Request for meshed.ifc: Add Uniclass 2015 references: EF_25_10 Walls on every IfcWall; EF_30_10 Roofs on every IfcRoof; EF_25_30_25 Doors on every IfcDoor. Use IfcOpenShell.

First a look at what the model holds.

```python
import ifcopenshell

model = ifcopenshell.open("meshed.ifc")
print(model.schema)
print("classifications:", [c.Name for c in model.by_type("IfcClassification")])
for ifc_class in ("IfcDoor", "IfcRoof", "IfcStair", "IfcWall", "IfcWindow"):
    print(ifc_class, len(model.by_type(ifc_class)))
```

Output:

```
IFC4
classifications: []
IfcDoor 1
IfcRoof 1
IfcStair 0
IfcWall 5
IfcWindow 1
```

```python
import ifcopenshell
import ifcopenshell.api.classification

model = ifcopenshell.open("meshed.ifc")

system = ifcopenshell.api.classification.add_classification(model, classification="Uniclass 2015")

codes = {
    "IfcWall": ("EF_25_10", "Walls"),
    "IfcRoof": ("EF_30_10", "Roofs"),
    "IfcDoor": ("EF_25_30_25", "Doors"),
}
for ifc_class, (code, name) in codes.items():
    products = model.by_type(ifc_class)
    ifcopenshell.api.classification.add_reference(
        model, products=products, classification=system, identification=code, name=name
    )
    print(code, len(products))

model.write("meshed_rev.ifc")
```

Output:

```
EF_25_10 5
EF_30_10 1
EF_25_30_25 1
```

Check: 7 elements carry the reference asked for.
